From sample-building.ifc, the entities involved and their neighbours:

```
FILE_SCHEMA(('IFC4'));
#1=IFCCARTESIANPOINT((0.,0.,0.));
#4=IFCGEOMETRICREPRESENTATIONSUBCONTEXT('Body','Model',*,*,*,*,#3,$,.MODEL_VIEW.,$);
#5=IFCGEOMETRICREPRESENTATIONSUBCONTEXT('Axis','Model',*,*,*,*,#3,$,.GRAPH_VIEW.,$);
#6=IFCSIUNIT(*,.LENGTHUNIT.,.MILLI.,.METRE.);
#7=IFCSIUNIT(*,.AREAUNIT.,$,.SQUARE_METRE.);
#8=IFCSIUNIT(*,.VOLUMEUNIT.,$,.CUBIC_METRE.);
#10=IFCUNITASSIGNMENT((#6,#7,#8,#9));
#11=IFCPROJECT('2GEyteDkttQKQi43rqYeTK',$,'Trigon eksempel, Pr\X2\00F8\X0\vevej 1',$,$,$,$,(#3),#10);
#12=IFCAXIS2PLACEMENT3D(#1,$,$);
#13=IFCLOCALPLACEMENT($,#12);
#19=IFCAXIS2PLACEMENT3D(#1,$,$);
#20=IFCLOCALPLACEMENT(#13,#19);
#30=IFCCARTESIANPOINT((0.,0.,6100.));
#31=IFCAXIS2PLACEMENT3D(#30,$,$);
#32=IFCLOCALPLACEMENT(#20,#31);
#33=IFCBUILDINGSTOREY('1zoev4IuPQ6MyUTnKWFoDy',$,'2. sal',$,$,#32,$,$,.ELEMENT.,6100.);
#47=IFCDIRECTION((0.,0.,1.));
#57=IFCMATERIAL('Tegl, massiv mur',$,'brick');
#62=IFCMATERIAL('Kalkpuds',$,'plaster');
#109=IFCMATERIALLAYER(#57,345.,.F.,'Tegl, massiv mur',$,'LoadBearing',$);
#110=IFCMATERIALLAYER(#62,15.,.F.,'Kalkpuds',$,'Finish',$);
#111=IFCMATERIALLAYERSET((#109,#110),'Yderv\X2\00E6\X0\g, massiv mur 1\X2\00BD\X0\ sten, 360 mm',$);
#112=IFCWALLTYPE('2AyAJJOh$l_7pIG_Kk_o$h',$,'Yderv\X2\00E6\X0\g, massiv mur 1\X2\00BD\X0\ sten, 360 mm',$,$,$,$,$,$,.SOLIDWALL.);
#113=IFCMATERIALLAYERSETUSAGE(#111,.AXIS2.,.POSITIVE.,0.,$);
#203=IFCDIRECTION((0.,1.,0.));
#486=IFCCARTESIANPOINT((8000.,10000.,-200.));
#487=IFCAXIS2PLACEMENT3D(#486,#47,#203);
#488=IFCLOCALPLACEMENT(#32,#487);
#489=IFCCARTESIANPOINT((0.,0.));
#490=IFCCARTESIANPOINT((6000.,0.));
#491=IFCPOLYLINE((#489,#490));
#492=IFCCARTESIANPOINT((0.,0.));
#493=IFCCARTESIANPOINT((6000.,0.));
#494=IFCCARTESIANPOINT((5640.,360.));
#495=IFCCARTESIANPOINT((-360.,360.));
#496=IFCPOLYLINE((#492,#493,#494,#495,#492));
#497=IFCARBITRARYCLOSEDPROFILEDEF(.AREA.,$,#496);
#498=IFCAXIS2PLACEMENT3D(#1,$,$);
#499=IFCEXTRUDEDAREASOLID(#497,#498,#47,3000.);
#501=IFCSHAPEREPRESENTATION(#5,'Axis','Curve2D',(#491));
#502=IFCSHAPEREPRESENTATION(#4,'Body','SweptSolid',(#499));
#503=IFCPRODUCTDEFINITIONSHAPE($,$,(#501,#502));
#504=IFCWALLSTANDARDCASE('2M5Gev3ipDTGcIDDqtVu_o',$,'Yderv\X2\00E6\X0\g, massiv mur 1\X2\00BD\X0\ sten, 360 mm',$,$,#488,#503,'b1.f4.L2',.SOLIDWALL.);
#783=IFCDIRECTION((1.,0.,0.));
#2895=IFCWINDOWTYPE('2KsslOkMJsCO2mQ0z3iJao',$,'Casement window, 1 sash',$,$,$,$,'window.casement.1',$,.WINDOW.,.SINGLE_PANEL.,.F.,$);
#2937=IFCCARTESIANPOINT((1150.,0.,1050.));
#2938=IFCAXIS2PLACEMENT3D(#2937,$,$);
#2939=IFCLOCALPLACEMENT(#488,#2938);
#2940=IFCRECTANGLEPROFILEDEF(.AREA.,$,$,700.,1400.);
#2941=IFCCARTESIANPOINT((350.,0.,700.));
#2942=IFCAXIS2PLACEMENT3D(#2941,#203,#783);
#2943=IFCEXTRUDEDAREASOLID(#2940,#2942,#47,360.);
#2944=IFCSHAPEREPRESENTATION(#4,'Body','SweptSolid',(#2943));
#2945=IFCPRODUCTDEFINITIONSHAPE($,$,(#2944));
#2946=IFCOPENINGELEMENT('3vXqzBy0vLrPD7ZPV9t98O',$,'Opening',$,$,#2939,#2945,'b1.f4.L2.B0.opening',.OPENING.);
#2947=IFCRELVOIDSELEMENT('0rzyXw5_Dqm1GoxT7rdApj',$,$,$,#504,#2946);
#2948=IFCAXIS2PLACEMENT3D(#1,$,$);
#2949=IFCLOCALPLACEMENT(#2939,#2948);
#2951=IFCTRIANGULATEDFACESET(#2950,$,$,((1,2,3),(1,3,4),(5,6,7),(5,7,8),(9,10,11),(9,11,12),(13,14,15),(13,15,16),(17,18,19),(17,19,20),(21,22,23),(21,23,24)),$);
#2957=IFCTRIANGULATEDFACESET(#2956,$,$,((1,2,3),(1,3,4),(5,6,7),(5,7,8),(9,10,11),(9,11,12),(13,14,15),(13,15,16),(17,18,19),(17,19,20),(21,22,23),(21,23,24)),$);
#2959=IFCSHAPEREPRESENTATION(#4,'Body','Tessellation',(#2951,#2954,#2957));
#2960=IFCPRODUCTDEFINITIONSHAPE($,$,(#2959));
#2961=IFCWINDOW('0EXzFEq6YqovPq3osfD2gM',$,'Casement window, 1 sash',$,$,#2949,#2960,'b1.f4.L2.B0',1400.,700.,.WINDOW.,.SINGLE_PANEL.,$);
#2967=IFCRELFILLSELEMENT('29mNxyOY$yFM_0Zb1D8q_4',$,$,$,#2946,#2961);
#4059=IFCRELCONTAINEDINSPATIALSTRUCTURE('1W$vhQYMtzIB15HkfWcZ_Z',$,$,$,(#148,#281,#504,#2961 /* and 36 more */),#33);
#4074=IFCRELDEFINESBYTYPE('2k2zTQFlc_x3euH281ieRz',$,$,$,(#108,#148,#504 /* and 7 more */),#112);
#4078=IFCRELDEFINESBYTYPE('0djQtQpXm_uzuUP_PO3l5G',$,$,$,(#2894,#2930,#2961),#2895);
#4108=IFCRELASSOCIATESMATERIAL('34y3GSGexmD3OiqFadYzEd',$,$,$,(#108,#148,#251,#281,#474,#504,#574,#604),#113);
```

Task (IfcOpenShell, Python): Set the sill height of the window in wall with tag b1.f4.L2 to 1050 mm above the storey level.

```python
import numpy as np
import ifcopenshell
import ifcopenshell.api.geometry
import ifcopenshell.geom
import ifcopenshell.util.element
import ifcopenshell.util.placement
import ifcopenshell.util.shape
import ifcopenshell.util.unit

model = ifcopenshell.open("sample-building.ifc")
unit_scale = ifcopenshell.util.unit.calculate_unit_scale(model)

window = model.by_guid("0EXzFEq6YqovPq3osfD2gM")
opening = window.FillsVoids[0].RelatingOpeningElement
storey = ifcopenshell.util.element.get_container(window, ifc_class="IfcBuildingStorey")
level = ifcopenshell.util.placement.get_local_placement(storey.ObjectPlacement)[2, 3]

# The opening's origin need not be at the sill, so measure its lowest point.
shape = ifcopenshell.geom.create_shape(ifcopenshell.geom.settings(), opening)
bottom = ifcopenshell.util.shape.get_shape_bottom_elevation(shape, shape.geometry) / unit_scale
dz = level + 1.05 / unit_scale - bottom

shift = np.array([0.0, 0.0, dz])
# The window is placed relative to its opening, so it follows when the opening moves.
matrix = ifcopenshell.util.placement.get_local_placement(opening.ObjectPlacement)
matrix[:3, 3] += shift
ifcopenshell.api.geometry.edit_object_placement(
    model, product=opening, matrix=matrix, is_si=False, should_transform_children=True
)

print(f"moved by {dz * unit_scale:+.3f} m")

model.write("sample-building_v2.ifc")
```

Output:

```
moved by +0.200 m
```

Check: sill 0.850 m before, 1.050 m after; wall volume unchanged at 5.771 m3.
